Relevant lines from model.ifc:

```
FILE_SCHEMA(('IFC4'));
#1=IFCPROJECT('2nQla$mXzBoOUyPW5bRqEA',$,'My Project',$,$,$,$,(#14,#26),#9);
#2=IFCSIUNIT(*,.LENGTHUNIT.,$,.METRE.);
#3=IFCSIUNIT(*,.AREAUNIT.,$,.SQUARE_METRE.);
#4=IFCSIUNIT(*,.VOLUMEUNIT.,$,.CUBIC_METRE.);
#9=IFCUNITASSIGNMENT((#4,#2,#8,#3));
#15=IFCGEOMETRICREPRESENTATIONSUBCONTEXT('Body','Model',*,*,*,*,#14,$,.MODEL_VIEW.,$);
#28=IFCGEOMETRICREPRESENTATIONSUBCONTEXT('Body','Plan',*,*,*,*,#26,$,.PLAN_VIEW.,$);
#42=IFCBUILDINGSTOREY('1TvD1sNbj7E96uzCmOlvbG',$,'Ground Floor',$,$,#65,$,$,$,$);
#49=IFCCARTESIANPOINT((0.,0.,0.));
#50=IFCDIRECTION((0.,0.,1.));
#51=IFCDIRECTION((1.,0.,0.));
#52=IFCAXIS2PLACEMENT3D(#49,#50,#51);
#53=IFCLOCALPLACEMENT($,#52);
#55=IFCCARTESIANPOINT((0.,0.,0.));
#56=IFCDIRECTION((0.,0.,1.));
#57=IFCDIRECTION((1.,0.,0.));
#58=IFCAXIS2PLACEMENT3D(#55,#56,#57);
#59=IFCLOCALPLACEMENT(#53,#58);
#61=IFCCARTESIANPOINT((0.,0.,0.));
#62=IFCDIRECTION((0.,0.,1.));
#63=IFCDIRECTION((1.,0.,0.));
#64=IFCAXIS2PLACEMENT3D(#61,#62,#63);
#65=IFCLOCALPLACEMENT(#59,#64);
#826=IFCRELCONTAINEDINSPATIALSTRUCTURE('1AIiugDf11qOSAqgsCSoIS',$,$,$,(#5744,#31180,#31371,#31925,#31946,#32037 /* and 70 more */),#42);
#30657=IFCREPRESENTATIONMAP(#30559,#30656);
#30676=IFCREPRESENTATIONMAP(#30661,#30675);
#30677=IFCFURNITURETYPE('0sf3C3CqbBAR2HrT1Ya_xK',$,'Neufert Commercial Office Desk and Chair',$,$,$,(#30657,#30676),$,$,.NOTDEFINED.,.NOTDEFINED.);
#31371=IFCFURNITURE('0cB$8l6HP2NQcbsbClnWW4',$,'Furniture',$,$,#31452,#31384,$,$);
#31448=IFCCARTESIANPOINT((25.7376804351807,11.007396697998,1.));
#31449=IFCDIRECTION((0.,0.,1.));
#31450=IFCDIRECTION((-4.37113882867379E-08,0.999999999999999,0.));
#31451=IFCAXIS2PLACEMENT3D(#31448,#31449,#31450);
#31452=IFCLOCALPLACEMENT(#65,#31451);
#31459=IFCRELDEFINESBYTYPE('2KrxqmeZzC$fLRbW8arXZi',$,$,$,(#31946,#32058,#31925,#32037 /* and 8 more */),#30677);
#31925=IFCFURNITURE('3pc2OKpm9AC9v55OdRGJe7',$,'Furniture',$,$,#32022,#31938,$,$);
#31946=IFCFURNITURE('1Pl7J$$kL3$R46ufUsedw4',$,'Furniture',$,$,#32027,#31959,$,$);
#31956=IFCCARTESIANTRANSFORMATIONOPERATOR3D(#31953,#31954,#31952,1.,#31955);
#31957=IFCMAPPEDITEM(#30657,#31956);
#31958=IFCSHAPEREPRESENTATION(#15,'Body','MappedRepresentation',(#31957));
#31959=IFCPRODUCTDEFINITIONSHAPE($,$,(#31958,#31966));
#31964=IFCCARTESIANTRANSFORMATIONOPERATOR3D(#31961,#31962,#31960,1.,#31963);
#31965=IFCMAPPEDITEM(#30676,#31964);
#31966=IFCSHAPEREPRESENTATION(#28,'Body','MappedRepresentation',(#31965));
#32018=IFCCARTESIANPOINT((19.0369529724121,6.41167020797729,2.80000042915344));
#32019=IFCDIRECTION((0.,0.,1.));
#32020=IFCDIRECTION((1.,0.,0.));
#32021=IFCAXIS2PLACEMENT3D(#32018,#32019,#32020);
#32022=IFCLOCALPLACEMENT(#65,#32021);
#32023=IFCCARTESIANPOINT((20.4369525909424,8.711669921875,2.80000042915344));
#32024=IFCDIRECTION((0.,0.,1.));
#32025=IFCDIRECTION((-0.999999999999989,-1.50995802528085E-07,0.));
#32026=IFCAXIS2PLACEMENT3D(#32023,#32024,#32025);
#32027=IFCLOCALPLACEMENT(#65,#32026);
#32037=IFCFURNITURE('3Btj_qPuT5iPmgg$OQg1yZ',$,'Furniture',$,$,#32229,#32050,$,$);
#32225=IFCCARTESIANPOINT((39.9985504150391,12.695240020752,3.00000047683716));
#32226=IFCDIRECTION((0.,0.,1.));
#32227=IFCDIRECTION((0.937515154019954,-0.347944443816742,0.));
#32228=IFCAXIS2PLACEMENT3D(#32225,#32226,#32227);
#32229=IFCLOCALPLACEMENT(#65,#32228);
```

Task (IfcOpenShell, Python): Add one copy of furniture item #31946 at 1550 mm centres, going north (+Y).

```python
import numpy as np
import ifcopenshell
import ifcopenshell.api.geometry
import ifcopenshell.api.root
import ifcopenshell.util.element
import ifcopenshell.util.placement

model = ifcopenshell.open("model.ifc")

source = model.by_id(31946)
base = ifcopenshell.util.placement.get_local_placement(source.ObjectPlacement)
step = np.array([0.0, 1.0, 0.0]) * 1.55

for i in range(1, 2):
    copy = ifcopenshell.api.root.copy_class(model, product=source)
    copy.Representation = ifcopenshell.util.element.copy_deep(
        model, source.Representation, exclude=["IfcGeometricRepresentationContext", "IfcRepresentationMap"]
    )
    matrix = base.copy()
    matrix[:3, 3] += i * step
    print("added at", matrix[:3, 3].round(3) + 0.0)
    ifcopenshell.api.geometry.edit_object_placement(model, product=copy, matrix=matrix, is_si=False)

model.write("model_rev.ifc")
```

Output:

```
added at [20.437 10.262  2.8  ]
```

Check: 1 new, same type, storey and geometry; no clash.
